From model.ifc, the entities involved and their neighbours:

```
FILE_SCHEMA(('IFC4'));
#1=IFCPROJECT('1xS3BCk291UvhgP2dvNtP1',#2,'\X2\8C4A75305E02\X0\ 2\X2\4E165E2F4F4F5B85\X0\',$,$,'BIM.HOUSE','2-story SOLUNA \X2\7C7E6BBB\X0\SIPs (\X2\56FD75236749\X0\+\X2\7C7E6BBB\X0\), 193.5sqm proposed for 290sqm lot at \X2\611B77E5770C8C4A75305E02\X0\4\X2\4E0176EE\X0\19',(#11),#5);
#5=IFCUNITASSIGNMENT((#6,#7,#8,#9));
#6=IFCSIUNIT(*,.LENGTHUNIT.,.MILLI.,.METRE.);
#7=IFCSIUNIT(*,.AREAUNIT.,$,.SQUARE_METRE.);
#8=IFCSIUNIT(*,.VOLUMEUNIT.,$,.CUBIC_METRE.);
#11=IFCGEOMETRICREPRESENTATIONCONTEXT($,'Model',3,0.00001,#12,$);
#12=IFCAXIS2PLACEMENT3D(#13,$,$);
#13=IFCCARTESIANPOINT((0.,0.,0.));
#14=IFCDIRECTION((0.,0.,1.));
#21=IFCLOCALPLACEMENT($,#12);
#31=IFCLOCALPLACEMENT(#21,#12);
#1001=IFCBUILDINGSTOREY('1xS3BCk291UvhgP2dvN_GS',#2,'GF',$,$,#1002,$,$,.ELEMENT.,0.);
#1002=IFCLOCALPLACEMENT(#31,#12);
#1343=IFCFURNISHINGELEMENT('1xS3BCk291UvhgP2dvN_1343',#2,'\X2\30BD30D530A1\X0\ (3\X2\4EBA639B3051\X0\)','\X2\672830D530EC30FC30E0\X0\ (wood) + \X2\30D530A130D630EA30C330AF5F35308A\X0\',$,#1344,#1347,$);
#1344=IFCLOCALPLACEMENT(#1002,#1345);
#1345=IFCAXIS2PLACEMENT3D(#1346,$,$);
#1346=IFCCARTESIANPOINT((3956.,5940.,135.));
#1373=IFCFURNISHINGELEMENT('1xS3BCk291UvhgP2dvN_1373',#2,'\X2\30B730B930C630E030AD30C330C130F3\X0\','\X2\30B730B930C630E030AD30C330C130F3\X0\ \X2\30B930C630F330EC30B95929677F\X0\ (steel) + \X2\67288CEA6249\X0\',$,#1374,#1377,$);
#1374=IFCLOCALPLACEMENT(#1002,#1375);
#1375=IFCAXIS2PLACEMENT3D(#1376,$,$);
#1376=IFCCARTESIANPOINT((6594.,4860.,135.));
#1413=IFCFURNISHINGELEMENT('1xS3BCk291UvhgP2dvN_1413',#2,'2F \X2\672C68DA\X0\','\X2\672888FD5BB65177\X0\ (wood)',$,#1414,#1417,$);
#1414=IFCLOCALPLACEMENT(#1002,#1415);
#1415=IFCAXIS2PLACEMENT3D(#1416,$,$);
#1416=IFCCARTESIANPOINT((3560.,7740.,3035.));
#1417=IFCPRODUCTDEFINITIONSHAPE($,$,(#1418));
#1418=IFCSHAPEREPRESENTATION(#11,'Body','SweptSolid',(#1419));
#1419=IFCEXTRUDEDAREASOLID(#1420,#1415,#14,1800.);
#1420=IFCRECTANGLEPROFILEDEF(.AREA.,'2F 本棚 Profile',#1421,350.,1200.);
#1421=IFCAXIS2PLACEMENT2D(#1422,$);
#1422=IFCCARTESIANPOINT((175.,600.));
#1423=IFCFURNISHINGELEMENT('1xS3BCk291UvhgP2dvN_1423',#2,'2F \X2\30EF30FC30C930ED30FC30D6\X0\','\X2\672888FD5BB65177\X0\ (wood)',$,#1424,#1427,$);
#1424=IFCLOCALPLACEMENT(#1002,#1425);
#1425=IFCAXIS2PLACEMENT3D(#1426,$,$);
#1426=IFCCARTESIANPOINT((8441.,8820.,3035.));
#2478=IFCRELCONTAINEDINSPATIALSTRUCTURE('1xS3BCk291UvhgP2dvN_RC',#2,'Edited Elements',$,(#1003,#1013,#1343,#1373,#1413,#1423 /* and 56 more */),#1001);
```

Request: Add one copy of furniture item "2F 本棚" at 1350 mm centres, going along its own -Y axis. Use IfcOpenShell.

```python
import ifcopenshell
import ifcopenshell.api.geometry
import ifcopenshell.api.root
import ifcopenshell.util.element
import ifcopenshell.util.placement
import ifcopenshell.util.unit

model = ifcopenshell.open("model.ifc")
unit_scale = ifcopenshell.util.unit.calculate_unit_scale(model)


def reuse_history(source, copy):
    """copy_class also copies each property set's owner history, people and application; keep the originals."""
    for rel in copy.IsDefinedBy:
        if rel.is_a("IfcRelDefinesByProperties") and (history := rel.RelatingPropertyDefinition.OwnerHistory):
            rel.RelatingPropertyDefinition.OwnerHistory = source.OwnerHistory
            ifcopenshell.util.element.remove_deep2(model, history)


source = model.by_guid("1xS3BCk291UvhgP2dvN_1413")
base = ifcopenshell.util.placement.get_local_placement(source.ObjectPlacement)
step = -base[:3, 1] * 1.35 / unit_scale

for i in range(1, 2):
    copy = ifcopenshell.api.root.copy_class(model, product=source)
    copy.Representation = ifcopenshell.util.element.copy_deep(
        model, source.Representation, exclude=["IfcGeometricRepresentationContext", "IfcRepresentationMap"]
    )
    reuse_history(source, copy)
    matrix = base.copy()
    matrix[:3, 3] += i * step
    print("added at", matrix[:3, 3].round(3) + 0.0)
    ifcopenshell.api.geometry.edit_object_placement(model, product=copy, matrix=matrix, is_si=False)

model.write("model-out.ifc")
```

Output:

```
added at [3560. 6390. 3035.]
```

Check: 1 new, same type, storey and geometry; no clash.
